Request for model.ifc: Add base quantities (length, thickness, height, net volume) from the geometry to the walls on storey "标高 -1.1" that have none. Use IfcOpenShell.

First a look at what the model holds.

```python
import ifcopenshell
import ifcopenshell.util.element
import ifcopenshell.util.unit

model = ifcopenshell.open("model.ifc")
print(model.schema)
for unit_type in ("LENGTHUNIT", "AREAUNIT", "VOLUMEUNIT"):
    print(unit_type, ifcopenshell.util.unit.calculate_unit_scale(model, unit_type))
storey = next(s for s in model.by_type("IfcBuildingStorey") if s.Name == "标高 -1.1")
walls = [e for e in ifcopenshell.util.element.get_decomposition(storey) if e.is_a("IfcWall")]
for e in sorted(walls, key=lambda e: e.id()):
    print(e.id(), e.is_a(), e.Name, list(ifcopenshell.util.element.get_psets(e, qtos_only=True)), sep=" | ")
```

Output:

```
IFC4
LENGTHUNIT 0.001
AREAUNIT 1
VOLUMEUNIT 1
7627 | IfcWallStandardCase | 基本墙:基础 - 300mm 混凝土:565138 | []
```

```python
import ifcopenshell
import ifcopenshell.api.pset
import ifcopenshell.geom
import ifcopenshell.util.element
import ifcopenshell.util.shape
import ifcopenshell.util.unit

model = ifcopenshell.open("model.ifc")
unit_scale = ifcopenshell.util.unit.calculate_unit_scale(model)
volume_scale = ifcopenshell.util.unit.calculate_unit_scale(model, "VOLUMEUNIT")
settings = ifcopenshell.geom.settings()

storey = next(s for s in model.by_type("IfcBuildingStorey") if s.Name == "标高 -1.1")
walls = [e for e in ifcopenshell.util.element.get_decomposition(storey) if e.is_a("IfcWall")]

for e in sorted(walls, key=lambda e: e.id()):
    if ifcopenshell.util.element.get_psets(e, qtos_only=True, should_inherit=False):
        continue
    # Geometry comes back in metres, in the element's own axes.
    shape = ifcopenshell.geom.create_shape(settings, e)
    values = {
        "Length": ifcopenshell.util.shape.get_x(shape.geometry) / unit_scale,
        "Width": ifcopenshell.util.shape.get_y(shape.geometry) / unit_scale,
        "Height": ifcopenshell.util.shape.get_z(shape.geometry) / unit_scale,
        "NetVolume": ifcopenshell.util.shape.get_volume(shape.geometry) / volume_scale,
    }
    qto = ifcopenshell.api.pset.add_qto(model, product=e, name="Qto_WallBaseQuantities")
    ifcopenshell.api.pset.edit_qto(model, qto=qto, properties=values)
    print(e.id(), {k: round(v, 3) for k, v in values.items()})

model.write("model_edited.ifc")
```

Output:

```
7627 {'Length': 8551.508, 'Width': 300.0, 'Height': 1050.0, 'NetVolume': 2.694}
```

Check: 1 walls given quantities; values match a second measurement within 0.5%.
